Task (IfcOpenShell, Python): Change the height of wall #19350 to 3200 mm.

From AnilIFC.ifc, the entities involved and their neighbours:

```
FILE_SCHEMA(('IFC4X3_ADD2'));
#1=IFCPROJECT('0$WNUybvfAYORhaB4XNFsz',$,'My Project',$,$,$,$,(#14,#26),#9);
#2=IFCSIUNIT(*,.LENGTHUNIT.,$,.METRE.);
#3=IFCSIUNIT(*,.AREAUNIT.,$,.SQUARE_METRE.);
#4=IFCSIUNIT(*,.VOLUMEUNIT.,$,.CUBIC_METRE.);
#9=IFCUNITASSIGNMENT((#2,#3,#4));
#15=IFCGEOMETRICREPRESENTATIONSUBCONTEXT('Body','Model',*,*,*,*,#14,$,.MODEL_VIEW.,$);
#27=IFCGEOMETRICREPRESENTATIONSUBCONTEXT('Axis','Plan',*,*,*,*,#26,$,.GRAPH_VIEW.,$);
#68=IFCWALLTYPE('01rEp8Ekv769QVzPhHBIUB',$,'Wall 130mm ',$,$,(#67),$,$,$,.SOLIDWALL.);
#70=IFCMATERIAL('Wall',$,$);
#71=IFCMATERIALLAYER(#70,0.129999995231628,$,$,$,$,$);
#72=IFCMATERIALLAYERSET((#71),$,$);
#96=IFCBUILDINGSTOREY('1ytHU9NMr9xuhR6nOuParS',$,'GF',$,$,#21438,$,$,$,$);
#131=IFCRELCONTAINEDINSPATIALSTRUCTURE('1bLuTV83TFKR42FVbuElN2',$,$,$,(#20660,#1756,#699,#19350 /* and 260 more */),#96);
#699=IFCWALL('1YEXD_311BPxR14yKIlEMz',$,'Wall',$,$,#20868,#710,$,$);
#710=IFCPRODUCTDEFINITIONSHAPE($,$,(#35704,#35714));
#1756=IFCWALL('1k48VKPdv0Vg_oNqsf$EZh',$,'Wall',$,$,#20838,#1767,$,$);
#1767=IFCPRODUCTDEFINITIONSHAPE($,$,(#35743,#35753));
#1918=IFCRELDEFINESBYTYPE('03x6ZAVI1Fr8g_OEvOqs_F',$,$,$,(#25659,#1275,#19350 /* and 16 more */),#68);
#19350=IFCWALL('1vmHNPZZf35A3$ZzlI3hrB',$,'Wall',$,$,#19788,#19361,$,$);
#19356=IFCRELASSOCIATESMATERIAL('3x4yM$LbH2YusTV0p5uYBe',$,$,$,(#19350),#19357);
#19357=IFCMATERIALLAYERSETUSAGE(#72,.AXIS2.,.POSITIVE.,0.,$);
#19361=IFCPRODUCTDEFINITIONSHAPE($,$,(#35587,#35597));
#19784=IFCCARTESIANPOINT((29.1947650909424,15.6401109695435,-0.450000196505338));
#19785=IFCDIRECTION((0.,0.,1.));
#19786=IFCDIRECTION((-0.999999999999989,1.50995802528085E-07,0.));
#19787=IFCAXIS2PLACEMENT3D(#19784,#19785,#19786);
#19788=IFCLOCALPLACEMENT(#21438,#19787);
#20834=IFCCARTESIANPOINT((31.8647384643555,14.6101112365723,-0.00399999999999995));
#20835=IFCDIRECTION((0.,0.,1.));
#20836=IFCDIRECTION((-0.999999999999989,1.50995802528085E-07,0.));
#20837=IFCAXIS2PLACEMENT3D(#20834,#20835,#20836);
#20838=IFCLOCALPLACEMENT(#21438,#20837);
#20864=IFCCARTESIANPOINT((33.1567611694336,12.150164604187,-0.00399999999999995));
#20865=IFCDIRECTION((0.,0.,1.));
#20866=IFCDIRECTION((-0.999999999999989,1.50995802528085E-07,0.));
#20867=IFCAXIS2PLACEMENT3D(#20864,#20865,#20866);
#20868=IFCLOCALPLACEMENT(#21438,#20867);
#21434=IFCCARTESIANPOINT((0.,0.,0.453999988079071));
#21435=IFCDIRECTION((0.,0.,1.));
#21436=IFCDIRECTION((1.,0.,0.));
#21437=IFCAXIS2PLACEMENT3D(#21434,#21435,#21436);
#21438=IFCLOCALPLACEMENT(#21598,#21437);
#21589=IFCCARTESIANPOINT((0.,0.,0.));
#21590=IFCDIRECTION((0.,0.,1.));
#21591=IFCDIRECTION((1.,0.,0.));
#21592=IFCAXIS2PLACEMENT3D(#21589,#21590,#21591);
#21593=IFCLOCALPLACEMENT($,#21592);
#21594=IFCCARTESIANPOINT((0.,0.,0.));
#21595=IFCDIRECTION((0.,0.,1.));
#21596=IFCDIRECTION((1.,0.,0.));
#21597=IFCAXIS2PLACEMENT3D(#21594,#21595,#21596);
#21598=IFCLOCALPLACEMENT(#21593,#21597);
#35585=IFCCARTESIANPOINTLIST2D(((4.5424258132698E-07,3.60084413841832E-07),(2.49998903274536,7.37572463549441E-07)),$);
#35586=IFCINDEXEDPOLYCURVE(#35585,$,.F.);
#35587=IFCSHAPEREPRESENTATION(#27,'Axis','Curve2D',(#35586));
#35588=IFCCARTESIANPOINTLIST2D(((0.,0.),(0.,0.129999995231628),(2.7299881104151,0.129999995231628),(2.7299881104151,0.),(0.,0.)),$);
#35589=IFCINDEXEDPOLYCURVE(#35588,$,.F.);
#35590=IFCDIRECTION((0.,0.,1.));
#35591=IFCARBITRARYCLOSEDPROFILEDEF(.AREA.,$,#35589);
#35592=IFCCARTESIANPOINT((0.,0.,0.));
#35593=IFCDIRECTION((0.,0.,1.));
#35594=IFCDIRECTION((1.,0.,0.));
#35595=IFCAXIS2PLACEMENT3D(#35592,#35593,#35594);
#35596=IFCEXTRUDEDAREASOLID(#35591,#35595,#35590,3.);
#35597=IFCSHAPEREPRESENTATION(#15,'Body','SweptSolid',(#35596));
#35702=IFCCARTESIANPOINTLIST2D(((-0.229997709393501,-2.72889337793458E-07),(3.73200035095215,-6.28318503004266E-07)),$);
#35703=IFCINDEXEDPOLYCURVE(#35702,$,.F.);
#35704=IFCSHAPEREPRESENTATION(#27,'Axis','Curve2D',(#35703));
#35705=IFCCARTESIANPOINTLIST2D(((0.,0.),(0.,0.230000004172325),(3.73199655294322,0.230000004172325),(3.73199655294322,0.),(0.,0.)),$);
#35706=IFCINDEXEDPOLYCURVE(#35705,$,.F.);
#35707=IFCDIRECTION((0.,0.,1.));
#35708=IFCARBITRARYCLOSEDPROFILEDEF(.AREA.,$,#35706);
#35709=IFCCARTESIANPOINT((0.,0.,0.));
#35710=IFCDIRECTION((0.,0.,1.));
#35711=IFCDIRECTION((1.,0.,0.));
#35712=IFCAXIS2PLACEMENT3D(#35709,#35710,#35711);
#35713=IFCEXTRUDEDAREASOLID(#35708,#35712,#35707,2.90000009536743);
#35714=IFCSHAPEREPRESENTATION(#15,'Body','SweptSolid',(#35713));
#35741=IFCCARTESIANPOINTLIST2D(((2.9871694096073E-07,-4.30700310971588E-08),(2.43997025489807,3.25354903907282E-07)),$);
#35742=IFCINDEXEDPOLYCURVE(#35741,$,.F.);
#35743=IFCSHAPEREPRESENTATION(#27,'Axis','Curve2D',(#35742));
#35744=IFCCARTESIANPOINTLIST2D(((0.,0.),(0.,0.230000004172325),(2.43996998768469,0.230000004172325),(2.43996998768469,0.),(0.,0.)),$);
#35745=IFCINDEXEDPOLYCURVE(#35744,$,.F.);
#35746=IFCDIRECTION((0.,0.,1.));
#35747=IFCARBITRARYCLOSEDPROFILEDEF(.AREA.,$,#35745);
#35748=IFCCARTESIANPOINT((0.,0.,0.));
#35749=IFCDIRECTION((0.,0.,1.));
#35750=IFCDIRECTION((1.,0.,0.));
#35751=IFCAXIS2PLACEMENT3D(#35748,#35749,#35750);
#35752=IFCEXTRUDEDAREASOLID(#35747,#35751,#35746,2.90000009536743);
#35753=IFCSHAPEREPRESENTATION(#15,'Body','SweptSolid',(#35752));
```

```python
import ifcopenshell
import ifcopenshell.geom
import ifcopenshell.util.representation
import ifcopenshell.util.shape
import ifcopenshell.util.unit

model = ifcopenshell.open("AnilIFC.ifc")
unit_scale = ifcopenshell.util.unit.calculate_unit_scale(model)
settings = ifcopenshell.geom.settings()


def volume(element):
    """Net volume in cubic metres, openings subtracted."""
    shape = ifcopenshell.geom.create_shape(settings, element)
    return ifcopenshell.util.shape.get_volume(shape.geometry)


wall = model.by_guid("1vmHNPZZf35A3$ZzlI3hrB")
before = volume(wall)

body = ifcopenshell.util.representation.get_representation(wall, "Model", "Body")
solid = body.Items[0]
old_height = solid.Depth
solid.Depth = 3.2 / unit_scale
after = volume(wall)

print(f"height {old_height:g} -> {solid.Depth:g}, volume {before:.3f} -> {after:.3f} m3")

model.write("AnilIFC_v2.ifc")
```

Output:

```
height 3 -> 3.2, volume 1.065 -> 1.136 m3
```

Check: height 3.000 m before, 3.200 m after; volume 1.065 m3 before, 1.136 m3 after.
